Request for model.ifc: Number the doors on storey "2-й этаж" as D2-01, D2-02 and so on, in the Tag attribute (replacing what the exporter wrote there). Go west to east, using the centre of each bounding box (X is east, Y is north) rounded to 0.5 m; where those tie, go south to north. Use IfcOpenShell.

First a look at what the model holds.

```python
import ifcopenshell
import ifcopenshell.util.element
import ifcopenshell.util.placement

model = ifcopenshell.open("model.ifc")
print(model.schema)
storey = next(s for s in model.by_type("IfcBuildingStorey") if s.Name == "2-й этаж")
doors = [e for e in ifcopenshell.util.element.get_decomposition(storey) if e.is_a("IfcDoor")]
for e in sorted(doors, key=lambda e: e.id()):
    origin = ifcopenshell.util.placement.get_local_placement(e.ObjectPlacement)[:3, 3]
    print(e.id(), e.Tag, e.Name, origin.round(2) + 0.0, sep=" | ")
```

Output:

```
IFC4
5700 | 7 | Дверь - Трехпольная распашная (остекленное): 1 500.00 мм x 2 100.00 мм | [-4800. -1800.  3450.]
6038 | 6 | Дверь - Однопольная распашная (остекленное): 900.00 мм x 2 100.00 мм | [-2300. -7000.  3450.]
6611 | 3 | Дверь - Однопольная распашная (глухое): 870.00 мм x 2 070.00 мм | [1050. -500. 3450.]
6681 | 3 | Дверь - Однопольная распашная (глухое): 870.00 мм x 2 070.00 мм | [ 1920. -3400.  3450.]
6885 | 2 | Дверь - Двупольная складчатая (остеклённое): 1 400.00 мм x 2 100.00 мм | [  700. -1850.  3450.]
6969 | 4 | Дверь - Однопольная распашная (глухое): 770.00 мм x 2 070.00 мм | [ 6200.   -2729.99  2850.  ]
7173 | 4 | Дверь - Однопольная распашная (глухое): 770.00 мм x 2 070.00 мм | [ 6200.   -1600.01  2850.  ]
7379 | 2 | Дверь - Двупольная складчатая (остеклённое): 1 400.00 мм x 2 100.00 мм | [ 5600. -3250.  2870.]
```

```python
import ifcopenshell
import ifcopenshell.geom
import ifcopenshell.util.element
import ifcopenshell.util.shape

model = ifcopenshell.open("model.ifc")
settings = ifcopenshell.geom.settings()
settings.set("use-world-coords", True)


def centre(element):
    shape = ifcopenshell.geom.create_shape(settings, element)
    return ifcopenshell.util.shape.get_bbox_centroid(shape.geometry)


storey = next(s for s in model.by_type("IfcBuildingStorey") if s.Name == "2-й этаж")
doors = [e for e in ifcopenshell.util.element.get_decomposition(storey) if e.is_a("IfcDoor")]

# Insertion points can sit at a corner or the storey origin, so sort by the geometry (in metres).
centres = {e: centre(e) for e in doors}
doors.sort(key=lambda e: (round(centres[e][0] / 0.5), centres[e][1]))

for i, e in enumerate(doors, start=1):
    number = f"D2-{i:02d}"
    e.Tag = number
    print(e.id(), number)

model.write("model_rev.ifc")
```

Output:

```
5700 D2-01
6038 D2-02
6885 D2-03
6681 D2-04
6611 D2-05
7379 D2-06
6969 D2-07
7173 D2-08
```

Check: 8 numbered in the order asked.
